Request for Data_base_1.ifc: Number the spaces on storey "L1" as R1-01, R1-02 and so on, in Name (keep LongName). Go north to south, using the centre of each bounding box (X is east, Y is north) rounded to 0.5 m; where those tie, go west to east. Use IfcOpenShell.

First a look at what the model holds.

```python
import ifcopenshell
import ifcopenshell.util.element
import ifcopenshell.util.placement

model = ifcopenshell.open("Data_base_1.ifc")
print(model.schema)
storey = next(s for s in model.by_type("IfcBuildingStorey") if s.Name == "L1")
spaces = [e for e in ifcopenshell.util.element.get_decomposition(storey) if e.is_a("IfcSpace")]
for e in sorted(spaces, key=lambda e: e.id()):
    origin = ifcopenshell.util.placement.get_local_placement(e.ObjectPlacement)[:3, 3]
    print(e.id(), e.Name, e.LongName, origin.round(2) + 0.0, sep=" | ")
```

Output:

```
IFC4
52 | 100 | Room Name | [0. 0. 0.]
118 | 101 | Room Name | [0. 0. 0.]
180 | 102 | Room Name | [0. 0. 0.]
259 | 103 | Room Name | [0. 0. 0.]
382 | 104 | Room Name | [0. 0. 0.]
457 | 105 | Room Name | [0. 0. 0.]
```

```python
import ifcopenshell
import ifcopenshell.geom
import ifcopenshell.util.element
import ifcopenshell.util.shape

model = ifcopenshell.open("Data_base_1.ifc")
settings = ifcopenshell.geom.settings()
settings.set("use-world-coords", True)


def centre(element):
    shape = ifcopenshell.geom.create_shape(settings, element)
    return ifcopenshell.util.shape.get_bbox_centroid(shape.geometry)


storey = next(s for s in model.by_type("IfcBuildingStorey") if s.Name == "L1")
spaces = [e for e in ifcopenshell.util.element.get_decomposition(storey) if e.is_a("IfcSpace")]

# Insertion points can sit at a corner or the storey origin, so sort by the geometry (in metres).
centres = {e: centre(e) for e in spaces}
spaces.sort(key=lambda e: (-round(centres[e][1] / 0.5), centres[e][0]))

for i, e in enumerate(spaces, start=1):
    number = f"R1-{i:02d}"
    e.Name = number
    print(e.id(), number)

model.write("Data_base_1_v2.ifc")
```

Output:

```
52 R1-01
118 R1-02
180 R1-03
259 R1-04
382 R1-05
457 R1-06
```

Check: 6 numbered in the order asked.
